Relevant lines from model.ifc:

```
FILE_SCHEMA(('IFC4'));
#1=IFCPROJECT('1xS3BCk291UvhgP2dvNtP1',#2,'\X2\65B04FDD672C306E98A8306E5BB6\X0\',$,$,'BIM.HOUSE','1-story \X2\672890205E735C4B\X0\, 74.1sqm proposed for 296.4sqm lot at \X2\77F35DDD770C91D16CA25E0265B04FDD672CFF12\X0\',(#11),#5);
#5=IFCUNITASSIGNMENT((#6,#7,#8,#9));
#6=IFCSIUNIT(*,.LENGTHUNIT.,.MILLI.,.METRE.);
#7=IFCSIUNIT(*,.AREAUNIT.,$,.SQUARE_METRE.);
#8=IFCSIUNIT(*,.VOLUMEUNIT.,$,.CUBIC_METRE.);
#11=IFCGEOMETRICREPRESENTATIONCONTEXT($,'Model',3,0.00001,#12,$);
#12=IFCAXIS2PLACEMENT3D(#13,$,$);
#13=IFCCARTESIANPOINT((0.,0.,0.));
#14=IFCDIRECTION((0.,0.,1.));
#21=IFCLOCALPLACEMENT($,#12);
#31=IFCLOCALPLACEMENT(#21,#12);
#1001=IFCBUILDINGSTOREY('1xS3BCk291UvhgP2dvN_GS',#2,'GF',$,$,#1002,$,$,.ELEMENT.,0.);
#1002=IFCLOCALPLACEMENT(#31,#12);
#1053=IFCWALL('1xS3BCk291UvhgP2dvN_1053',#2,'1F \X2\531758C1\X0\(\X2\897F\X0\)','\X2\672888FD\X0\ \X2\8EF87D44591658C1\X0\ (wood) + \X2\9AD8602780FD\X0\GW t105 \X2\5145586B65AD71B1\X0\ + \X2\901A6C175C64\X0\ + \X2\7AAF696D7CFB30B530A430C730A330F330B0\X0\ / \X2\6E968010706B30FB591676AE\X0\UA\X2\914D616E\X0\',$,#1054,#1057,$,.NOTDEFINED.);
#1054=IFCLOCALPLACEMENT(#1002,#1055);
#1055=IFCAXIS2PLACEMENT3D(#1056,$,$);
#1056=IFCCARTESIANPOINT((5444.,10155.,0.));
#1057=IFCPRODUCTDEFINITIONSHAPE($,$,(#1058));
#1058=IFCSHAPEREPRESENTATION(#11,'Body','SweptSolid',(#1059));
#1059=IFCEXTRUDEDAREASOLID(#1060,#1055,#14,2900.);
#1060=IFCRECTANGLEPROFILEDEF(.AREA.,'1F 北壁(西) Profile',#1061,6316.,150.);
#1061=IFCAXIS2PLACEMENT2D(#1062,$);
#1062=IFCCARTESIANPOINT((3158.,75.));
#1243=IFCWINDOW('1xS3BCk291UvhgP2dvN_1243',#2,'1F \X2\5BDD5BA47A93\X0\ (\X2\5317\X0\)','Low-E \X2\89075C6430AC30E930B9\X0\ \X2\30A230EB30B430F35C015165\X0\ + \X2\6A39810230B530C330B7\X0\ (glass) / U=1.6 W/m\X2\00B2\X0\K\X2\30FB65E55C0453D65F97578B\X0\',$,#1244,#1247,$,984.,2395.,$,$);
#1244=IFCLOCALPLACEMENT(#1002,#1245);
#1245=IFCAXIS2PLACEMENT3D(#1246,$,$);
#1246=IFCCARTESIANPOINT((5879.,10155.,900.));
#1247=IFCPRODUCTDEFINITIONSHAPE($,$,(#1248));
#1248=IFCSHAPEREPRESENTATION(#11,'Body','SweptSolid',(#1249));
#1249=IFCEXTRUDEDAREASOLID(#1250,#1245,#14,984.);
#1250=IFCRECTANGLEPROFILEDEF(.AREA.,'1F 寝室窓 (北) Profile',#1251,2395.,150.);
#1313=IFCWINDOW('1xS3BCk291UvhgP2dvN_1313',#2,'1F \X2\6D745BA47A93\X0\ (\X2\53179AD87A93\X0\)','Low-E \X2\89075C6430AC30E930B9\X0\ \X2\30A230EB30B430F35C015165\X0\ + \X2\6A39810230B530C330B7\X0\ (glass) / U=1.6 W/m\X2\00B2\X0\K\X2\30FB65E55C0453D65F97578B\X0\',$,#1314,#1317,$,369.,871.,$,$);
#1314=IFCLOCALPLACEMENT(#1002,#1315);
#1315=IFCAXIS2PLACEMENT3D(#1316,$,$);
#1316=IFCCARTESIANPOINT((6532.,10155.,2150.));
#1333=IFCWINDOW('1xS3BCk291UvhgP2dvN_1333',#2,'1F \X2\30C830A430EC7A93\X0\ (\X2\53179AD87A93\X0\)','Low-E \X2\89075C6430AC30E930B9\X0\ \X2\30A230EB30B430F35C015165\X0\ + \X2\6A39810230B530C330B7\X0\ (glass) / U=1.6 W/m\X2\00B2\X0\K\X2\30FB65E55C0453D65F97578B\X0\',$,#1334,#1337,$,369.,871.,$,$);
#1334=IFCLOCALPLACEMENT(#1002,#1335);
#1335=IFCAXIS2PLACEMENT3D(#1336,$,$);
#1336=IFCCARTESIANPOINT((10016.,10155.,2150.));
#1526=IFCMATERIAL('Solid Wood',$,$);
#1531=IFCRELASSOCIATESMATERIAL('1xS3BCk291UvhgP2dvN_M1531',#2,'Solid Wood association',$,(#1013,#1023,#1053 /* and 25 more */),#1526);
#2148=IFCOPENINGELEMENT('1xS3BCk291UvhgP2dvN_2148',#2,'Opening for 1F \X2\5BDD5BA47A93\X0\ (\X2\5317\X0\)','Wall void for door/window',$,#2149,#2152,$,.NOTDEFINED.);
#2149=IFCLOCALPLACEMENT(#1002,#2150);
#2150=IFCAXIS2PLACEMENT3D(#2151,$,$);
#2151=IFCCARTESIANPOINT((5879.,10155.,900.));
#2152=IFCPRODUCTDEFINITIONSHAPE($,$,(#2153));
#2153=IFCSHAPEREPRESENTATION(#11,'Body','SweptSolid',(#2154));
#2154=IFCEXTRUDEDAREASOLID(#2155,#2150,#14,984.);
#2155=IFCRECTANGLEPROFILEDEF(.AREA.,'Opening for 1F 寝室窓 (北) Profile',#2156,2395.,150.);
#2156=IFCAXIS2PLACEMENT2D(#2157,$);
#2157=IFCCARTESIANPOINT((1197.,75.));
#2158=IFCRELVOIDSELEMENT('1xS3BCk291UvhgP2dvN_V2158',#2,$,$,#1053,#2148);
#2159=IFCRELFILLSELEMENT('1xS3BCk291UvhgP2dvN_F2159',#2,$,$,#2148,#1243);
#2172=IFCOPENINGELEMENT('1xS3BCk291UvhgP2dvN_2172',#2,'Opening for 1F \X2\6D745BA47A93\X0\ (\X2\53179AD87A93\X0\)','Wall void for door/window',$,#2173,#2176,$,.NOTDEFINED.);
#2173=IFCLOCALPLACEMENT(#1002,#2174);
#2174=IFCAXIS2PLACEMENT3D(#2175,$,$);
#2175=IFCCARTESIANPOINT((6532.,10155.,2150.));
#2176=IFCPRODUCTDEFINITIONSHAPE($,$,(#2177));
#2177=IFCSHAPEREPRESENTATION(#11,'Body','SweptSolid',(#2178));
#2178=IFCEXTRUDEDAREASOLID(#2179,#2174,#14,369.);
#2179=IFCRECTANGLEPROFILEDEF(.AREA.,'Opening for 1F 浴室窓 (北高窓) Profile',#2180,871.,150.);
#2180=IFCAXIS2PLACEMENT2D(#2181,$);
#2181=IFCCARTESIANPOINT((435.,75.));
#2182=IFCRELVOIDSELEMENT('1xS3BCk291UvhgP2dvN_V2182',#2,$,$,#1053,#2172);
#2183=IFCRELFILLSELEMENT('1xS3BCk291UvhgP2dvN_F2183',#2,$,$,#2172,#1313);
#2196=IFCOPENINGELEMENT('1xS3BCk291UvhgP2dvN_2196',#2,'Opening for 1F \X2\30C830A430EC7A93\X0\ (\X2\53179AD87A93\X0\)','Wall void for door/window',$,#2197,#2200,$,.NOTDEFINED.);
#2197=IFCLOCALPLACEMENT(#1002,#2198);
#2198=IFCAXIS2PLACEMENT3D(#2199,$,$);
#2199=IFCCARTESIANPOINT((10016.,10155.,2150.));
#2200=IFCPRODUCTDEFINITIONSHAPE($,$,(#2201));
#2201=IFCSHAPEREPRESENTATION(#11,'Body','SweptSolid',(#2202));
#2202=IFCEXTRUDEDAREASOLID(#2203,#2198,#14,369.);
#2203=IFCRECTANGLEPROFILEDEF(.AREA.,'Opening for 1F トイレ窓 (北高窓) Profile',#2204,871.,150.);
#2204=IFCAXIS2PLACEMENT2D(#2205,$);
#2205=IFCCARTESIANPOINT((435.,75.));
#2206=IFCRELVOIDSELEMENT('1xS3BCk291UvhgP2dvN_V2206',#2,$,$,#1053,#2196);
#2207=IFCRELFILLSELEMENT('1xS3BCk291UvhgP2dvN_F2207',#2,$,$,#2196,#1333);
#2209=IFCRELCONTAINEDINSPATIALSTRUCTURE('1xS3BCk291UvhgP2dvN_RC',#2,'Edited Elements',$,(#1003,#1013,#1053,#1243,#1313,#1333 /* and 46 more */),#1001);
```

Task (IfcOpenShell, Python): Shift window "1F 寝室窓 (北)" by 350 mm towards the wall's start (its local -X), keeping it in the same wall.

```python
import ifcopenshell
import ifcopenshell.api.geometry
import ifcopenshell.util.placement
import ifcopenshell.util.unit

model = ifcopenshell.open("model.ifc")
unit_scale = ifcopenshell.util.unit.calculate_unit_scale(model)

window = model.by_guid("1xS3BCk291UvhgP2dvN_1243")
opening = window.FillsVoids[0].RelatingOpeningElement
wall = opening.VoidsElements[0].RelatingBuildingElement

wall_matrix = ifcopenshell.util.placement.get_local_placement(wall.ObjectPlacement)
shift = wall_matrix[:3, 0] * -0.35 / unit_scale
before = ifcopenshell.util.placement.get_local_placement(window.ObjectPlacement)[:3, 3].copy()

# The window is not placed relative to its opening, so move both.
for product in (opening, window):
    matrix = ifcopenshell.util.placement.get_local_placement(product.ObjectPlacement)
    matrix[:3, 3] += shift
    ifcopenshell.api.geometry.edit_object_placement(model, product=product, matrix=matrix, is_si=False)

after = ifcopenshell.util.placement.get_local_placement(window.ObjectPlacement)[:3, 3]
print("window moved by", (after - before).round(3) + 0.0)

model.write("model_v2.ifc")
```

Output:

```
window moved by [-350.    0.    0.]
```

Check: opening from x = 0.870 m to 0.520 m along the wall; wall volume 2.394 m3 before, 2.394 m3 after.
